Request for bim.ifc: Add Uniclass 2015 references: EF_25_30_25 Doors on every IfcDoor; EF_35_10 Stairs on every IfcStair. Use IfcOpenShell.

First a look at what the model holds.

```python
import ifcopenshell

model = ifcopenshell.open("bim.ifc")
print(model.schema)
print("classifications:", [c.Name for c in model.by_type("IfcClassification")])
for ifc_class in ("IfcDoor", "IfcRoof", "IfcStair", "IfcWall", "IfcWindow"):
    print(ifc_class, len(model.by_type(ifc_class)))
```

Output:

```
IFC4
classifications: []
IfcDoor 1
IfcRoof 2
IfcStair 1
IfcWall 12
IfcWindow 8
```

```python
import ifcopenshell
import ifcopenshell.api.classification

model = ifcopenshell.open("bim.ifc")

system = ifcopenshell.api.classification.add_classification(model, classification="Uniclass 2015")

codes = {
    "IfcDoor": ("EF_25_30_25", "Doors"),
    "IfcStair": ("EF_35_10", "Stairs"),
}
for ifc_class, (code, name) in codes.items():
    products = model.by_type(ifc_class)
    ifcopenshell.api.classification.add_reference(
        model, products=products, classification=system, identification=code, name=name
    )
    print(code, len(products))

model.write("bim_edited.ifc")
```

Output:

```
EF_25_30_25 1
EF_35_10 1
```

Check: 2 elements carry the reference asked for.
